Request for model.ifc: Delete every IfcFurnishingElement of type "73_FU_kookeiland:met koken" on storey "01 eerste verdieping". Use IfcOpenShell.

First a look at what the model holds.

```python
import ifcopenshell
import ifcopenshell.util.element

model = ifcopenshell.open("model.ifc")
print(model.schema)
storey = next(s for s in model.by_type("IfcBuildingStorey") if s.Name == "01 eerste verdieping")
furniture = [e for e in ifcopenshell.util.element.get_decomposition(storey) if e.is_a("IfcFurnishingElement")]
seen = {}
for e in furniture:
    element_type = ifcopenshell.util.element.get_type(e)
    name = element_type.Name if element_type not in (None, e) else None
    seen[name] = seen.get(name, 0) + 1
for name, count in sorted(seen.items(), key=str):
    print(count, "x", name)
```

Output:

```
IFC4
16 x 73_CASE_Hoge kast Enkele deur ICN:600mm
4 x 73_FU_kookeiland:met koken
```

```python
import ifcopenshell
import ifcopenshell.api.root
import ifcopenshell.util.element

model = ifcopenshell.open("model.ifc")

storey = next(s for s in model.by_type("IfcBuildingStorey") if s.Name == "01 eerste verdieping")
furniture = [e for e in ifcopenshell.util.element.get_decomposition(storey) if e.is_a("IfcFurnishingElement")]
targets = [e for e in furniture if (t := ifcopenshell.util.element.get_type(e)) not in (None, e) and t.Name == "73_FU_kookeiland:met koken"]

for e in targets:
    ifcopenshell.api.root.remove_product(model, product=e)
print(len(targets), "removed")

model.write("model_rev.ifc")
```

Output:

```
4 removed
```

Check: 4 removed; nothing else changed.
